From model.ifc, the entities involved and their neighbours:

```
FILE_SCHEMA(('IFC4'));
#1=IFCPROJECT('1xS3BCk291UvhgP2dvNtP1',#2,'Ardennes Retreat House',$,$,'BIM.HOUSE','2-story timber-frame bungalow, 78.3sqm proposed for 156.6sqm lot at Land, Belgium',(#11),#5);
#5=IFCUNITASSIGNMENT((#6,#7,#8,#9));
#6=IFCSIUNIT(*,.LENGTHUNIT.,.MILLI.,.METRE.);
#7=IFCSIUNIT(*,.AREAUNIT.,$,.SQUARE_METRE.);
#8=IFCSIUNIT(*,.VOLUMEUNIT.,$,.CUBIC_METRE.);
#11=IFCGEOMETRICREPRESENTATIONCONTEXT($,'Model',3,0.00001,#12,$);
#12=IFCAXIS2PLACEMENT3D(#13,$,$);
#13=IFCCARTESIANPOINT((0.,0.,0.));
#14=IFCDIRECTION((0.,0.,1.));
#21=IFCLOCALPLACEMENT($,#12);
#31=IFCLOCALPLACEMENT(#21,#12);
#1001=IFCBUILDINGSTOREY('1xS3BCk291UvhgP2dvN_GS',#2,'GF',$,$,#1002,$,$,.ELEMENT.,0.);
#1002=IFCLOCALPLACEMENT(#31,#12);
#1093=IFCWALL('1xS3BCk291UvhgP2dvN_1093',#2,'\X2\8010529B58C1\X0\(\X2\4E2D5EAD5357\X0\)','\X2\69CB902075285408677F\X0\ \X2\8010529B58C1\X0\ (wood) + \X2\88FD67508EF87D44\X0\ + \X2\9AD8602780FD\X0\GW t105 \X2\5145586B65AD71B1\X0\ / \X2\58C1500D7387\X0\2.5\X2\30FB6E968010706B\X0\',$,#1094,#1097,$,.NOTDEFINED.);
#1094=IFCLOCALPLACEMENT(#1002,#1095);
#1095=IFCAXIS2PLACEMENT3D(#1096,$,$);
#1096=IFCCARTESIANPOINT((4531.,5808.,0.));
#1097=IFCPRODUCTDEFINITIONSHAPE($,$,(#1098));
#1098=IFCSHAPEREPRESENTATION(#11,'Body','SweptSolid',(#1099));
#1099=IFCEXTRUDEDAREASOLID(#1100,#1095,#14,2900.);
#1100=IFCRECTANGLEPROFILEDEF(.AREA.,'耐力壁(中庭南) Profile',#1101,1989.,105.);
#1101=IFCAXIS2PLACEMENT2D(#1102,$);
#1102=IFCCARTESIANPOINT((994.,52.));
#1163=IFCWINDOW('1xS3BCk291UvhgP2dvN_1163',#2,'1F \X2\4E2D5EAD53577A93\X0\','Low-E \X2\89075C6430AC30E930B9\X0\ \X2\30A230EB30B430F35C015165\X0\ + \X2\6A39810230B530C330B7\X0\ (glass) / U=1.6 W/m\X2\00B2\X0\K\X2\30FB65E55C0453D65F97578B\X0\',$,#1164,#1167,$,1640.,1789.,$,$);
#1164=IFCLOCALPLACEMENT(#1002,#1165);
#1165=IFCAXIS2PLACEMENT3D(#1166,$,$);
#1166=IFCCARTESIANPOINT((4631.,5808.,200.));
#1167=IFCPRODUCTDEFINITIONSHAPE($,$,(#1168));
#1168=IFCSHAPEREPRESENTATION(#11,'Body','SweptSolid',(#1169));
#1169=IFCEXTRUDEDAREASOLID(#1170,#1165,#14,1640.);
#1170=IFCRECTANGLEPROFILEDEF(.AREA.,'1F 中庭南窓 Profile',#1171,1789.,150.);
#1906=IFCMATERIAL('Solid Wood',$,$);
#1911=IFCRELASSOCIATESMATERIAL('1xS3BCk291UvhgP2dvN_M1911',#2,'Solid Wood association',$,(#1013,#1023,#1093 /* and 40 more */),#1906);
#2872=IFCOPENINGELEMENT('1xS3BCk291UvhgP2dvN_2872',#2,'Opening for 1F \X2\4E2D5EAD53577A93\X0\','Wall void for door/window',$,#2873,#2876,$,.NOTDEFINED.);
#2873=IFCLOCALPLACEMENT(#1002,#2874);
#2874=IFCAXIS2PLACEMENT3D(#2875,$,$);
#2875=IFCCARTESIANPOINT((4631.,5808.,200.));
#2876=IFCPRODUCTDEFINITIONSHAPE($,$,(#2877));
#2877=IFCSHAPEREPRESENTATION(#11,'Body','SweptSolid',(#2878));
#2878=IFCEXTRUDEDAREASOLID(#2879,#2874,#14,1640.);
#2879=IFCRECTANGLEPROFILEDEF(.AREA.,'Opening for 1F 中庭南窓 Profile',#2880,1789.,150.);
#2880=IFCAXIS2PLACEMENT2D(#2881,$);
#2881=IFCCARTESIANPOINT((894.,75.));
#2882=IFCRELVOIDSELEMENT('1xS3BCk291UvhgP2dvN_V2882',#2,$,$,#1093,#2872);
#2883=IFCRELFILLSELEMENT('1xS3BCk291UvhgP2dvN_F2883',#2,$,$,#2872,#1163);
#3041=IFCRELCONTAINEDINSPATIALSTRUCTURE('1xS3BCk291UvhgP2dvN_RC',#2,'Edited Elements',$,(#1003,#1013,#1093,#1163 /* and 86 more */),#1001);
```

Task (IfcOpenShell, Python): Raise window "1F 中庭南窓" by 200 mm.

```python
import numpy as np
import ifcopenshell
import ifcopenshell.api.geometry
import ifcopenshell.util.placement
import ifcopenshell.util.unit

model = ifcopenshell.open("model.ifc")
unit_scale = ifcopenshell.util.unit.calculate_unit_scale(model)

window = model.by_id(1163)
opening = window.FillsVoids[0].RelatingOpeningElement
dz = 0.2 / unit_scale

shift = np.array([0.0, 0.0, dz])
# The window is not placed relative to its opening, so move both.
for product in (opening, window):
    matrix = ifcopenshell.util.placement.get_local_placement(product.ObjectPlacement)
    matrix[:3, 3] += shift
    ifcopenshell.api.geometry.edit_object_placement(model, product=product, matrix=matrix, is_si=False)

print(f"moved by {dz * unit_scale:+.3f} m")

model.write("model_updated.ifc")
```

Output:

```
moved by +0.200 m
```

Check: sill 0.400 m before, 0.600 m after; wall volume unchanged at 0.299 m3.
